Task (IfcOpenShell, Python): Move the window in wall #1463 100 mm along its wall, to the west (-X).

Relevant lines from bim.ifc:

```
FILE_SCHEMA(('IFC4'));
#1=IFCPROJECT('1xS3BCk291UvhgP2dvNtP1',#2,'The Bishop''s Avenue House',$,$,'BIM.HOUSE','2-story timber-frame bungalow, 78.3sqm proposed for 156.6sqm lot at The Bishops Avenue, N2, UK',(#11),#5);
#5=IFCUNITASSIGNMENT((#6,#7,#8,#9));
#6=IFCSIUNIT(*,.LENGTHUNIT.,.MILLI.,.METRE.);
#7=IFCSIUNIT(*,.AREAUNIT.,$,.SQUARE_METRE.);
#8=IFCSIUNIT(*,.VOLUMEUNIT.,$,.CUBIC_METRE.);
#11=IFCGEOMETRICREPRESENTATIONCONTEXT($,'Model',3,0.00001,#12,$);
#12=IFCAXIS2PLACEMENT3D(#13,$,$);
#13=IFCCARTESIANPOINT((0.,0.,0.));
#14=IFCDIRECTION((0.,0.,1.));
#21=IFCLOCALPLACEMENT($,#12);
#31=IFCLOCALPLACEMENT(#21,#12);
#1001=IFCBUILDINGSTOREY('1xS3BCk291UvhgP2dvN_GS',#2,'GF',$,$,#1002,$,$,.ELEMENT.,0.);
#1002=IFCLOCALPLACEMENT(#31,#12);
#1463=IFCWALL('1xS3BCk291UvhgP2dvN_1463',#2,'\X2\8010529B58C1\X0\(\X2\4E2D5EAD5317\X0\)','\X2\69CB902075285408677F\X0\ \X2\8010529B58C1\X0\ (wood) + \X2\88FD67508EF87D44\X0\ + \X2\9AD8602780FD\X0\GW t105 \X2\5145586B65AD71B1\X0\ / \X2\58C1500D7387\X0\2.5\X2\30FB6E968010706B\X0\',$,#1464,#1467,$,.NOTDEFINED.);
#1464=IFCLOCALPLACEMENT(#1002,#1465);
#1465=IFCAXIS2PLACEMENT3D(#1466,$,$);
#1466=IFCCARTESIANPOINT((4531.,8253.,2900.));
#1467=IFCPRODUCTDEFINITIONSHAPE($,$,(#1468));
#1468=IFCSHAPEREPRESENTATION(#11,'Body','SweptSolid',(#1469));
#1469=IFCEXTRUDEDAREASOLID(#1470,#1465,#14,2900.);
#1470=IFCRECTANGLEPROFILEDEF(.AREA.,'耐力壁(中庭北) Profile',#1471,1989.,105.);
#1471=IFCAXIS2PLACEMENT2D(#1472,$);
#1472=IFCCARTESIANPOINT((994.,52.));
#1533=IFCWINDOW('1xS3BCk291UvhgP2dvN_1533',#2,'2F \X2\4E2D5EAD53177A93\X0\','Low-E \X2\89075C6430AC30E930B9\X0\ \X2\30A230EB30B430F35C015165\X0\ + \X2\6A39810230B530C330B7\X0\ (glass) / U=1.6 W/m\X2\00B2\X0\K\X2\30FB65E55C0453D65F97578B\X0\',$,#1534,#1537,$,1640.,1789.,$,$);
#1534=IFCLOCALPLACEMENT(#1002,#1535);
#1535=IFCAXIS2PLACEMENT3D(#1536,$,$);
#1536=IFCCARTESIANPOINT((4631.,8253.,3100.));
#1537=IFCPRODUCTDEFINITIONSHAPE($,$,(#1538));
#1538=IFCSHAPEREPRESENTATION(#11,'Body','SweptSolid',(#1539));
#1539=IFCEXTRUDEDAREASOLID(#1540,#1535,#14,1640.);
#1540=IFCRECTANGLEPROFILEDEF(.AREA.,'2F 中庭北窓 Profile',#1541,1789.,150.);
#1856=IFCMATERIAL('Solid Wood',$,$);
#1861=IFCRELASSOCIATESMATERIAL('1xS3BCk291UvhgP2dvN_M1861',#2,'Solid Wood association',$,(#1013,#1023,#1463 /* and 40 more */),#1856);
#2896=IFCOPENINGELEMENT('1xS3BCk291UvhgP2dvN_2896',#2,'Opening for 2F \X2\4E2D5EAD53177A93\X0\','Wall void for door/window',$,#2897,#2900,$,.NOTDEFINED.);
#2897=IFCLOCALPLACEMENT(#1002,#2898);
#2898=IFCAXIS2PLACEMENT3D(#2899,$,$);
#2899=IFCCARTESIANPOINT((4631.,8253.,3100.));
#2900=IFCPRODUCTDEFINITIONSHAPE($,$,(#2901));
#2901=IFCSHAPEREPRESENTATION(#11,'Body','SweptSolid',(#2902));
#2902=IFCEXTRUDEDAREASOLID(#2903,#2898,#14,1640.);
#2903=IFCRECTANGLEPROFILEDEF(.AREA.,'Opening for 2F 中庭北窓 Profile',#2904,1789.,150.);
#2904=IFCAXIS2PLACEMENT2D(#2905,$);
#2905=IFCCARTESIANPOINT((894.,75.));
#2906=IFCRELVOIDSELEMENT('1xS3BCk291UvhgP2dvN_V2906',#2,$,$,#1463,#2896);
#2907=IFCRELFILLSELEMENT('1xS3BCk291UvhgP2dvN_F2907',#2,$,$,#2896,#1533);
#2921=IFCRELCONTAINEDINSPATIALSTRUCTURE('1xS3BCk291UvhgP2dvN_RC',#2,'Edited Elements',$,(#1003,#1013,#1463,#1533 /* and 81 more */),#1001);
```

```python
import ifcopenshell
import ifcopenshell.api.geometry
import ifcopenshell.util.placement

model = ifcopenshell.open("bim.ifc")

window = model.by_guid("1xS3BCk291UvhgP2dvN_1533")
opening = window.FillsVoids[0].RelatingOpeningElement
wall = opening.VoidsElements[0].RelatingBuildingElement

wall_matrix = ifcopenshell.util.placement.get_local_placement(wall.ObjectPlacement)
shift = wall_matrix[:3, 0] * -100.0
before = ifcopenshell.util.placement.get_local_placement(window.ObjectPlacement)[:3, 3].copy()

# The window is not placed relative to its opening, so move both.
for product in (opening, window):
    matrix = ifcopenshell.util.placement.get_local_placement(product.ObjectPlacement)
    matrix[:3, 3] += shift
    ifcopenshell.api.geometry.edit_object_placement(model, product=product, matrix=matrix, is_si=False)

after = ifcopenshell.util.placement.get_local_placement(window.ObjectPlacement)[:3, 3]
print("window moved by", (after - before).round(3) + 0.0)

model.write("bim_updated.ifc")
```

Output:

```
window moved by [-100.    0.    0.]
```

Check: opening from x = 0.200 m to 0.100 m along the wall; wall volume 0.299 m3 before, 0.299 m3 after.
